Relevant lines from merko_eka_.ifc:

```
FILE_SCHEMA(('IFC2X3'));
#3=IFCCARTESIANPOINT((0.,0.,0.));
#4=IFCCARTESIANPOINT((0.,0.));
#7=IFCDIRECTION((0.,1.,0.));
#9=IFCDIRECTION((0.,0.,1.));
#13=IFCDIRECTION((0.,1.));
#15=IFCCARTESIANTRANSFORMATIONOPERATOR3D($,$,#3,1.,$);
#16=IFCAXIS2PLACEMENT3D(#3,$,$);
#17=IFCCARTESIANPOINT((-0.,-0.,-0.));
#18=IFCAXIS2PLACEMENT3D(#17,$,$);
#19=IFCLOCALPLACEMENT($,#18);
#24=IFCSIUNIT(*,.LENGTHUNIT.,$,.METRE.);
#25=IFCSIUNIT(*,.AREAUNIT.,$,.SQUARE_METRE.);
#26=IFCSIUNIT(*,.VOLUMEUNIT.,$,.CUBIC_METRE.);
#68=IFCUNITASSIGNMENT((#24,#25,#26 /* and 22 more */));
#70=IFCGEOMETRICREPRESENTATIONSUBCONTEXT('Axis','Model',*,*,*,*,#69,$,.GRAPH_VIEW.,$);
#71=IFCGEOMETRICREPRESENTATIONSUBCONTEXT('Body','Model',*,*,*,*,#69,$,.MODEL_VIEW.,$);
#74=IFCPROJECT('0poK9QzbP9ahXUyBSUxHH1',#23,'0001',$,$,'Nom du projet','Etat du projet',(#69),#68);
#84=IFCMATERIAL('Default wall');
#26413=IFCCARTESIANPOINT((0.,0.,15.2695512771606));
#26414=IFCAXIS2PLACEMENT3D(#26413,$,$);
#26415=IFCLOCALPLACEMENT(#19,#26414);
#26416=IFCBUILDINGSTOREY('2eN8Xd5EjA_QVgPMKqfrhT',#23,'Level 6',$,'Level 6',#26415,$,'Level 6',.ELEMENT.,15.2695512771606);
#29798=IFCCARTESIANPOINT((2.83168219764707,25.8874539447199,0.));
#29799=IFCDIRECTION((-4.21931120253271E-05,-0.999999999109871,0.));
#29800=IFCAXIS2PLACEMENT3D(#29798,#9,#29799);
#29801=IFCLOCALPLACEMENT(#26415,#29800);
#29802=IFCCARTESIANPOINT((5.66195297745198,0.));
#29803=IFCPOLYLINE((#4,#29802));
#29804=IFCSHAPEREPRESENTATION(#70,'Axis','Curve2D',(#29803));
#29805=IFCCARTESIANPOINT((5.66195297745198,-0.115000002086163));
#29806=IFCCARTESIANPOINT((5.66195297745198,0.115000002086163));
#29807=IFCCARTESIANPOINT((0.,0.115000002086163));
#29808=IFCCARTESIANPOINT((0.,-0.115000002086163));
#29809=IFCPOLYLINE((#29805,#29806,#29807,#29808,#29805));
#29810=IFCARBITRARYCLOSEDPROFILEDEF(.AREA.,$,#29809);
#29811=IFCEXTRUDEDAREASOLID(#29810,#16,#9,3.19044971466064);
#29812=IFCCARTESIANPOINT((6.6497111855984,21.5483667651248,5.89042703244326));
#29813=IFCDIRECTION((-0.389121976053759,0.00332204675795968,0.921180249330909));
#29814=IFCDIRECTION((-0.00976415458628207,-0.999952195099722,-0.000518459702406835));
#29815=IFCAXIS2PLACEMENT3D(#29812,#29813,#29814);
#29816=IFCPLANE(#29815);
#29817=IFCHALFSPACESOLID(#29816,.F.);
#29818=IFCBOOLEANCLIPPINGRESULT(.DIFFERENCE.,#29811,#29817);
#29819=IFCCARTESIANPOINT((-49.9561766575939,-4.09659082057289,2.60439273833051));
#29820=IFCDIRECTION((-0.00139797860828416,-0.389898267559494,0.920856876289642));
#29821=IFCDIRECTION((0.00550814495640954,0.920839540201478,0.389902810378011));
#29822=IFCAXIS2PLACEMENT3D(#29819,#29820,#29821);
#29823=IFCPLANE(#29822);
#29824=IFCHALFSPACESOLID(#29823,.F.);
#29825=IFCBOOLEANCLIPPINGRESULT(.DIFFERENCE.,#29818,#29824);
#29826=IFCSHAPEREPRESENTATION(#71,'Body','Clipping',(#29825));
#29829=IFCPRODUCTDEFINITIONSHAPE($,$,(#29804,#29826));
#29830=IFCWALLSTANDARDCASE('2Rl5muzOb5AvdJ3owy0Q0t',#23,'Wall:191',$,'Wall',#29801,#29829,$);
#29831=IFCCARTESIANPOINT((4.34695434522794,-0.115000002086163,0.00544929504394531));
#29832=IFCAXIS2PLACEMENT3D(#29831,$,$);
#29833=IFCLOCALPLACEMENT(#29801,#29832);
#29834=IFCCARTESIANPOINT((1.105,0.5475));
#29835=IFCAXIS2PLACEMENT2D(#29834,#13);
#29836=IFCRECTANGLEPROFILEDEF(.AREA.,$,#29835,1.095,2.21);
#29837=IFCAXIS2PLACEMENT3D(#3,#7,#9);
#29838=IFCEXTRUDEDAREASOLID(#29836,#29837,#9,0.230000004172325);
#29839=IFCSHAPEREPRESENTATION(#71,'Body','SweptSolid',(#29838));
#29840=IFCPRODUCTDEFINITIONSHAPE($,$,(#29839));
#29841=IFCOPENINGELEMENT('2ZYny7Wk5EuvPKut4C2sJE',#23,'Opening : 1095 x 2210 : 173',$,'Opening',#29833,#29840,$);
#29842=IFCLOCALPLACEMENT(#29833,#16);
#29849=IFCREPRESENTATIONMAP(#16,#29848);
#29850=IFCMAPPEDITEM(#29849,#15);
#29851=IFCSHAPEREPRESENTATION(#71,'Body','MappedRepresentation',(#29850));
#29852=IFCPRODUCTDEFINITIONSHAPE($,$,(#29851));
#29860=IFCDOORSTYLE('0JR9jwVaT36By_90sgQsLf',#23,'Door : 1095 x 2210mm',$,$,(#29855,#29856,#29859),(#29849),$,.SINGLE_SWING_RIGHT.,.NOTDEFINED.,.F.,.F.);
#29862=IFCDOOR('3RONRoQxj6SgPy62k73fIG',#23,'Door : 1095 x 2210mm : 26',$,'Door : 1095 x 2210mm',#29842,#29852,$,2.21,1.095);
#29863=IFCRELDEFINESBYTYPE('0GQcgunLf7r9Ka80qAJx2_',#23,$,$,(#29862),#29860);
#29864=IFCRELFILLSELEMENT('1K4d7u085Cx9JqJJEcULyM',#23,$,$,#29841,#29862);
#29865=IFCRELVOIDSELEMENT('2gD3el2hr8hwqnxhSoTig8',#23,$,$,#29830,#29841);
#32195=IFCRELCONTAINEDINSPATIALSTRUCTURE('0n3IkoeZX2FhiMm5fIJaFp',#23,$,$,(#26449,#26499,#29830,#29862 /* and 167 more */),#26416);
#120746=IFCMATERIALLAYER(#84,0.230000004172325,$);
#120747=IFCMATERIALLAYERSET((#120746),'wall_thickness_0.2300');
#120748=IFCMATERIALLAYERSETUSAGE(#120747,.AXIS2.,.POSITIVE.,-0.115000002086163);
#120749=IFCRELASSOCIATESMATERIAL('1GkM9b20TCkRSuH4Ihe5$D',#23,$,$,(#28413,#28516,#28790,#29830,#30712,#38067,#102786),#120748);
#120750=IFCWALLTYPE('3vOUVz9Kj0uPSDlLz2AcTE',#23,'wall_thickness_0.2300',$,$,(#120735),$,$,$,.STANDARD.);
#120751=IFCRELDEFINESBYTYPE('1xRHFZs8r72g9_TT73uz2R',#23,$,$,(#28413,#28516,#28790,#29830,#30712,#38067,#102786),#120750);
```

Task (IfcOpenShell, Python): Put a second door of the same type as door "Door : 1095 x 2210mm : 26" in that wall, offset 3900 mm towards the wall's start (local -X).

```python
import ifcopenshell
import ifcopenshell.api.feature
import ifcopenshell.api.geometry
import ifcopenshell.api.root
import ifcopenshell.geom
import ifcopenshell.util.element
import ifcopenshell.util.placement
import ifcopenshell.util.shape
import ifcopenshell.util.unit

model = ifcopenshell.open("merko_eka_.ifc")
unit_scale = ifcopenshell.util.unit.calculate_unit_scale(model)
settings = ifcopenshell.geom.settings()


def volume(element):
    """Net volume in cubic metres, openings subtracted."""
    shape = ifcopenshell.geom.create_shape(settings, element)
    return ifcopenshell.util.shape.get_volume(shape.geometry)


door = model.by_guid("3RONRoQxj6SgPy62k73fIG")
opening = door.FillsVoids[0].RelatingOpeningElement
wall = opening.VoidsElements[0].RelatingBuildingElement
before = volume(wall)
shift = ifcopenshell.util.placement.get_local_placement(wall.ObjectPlacement)[:3, 0] * -3.9 / unit_scale

# copy_class copies the void relationship, type, container and properties, but no geometry.
new_opening = ifcopenshell.api.root.copy_class(model, product=opening)
new_opening.Representation = ifcopenshell.util.element.copy_deep(
    model, opening.Representation, exclude=["IfcGeometricRepresentationContext", "IfcRepresentationMap"]
)
new_opening.Name = "Opening : 1095 x 2210"
new_door = ifcopenshell.api.root.copy_class(model, product=door)
new_door.Representation = ifcopenshell.util.element.copy_deep(
    model, door.Representation, exclude=["IfcGeometricRepresentationContext", "IfcRepresentationMap"]
)
new_door.Name = "Door : 1095 x 2210mm"
fills = ifcopenshell.api.feature.add_filling(model, opening=new_opening, element=new_door)
fills.OwnerHistory = new_door.OwnerHistory  # required in IFC2X3

for old, new in ((opening, new_opening), (door, new_door)):
    matrix = ifcopenshell.util.placement.get_local_placement(old.ObjectPlacement)
    matrix[:3, 3] += shift
    ifcopenshell.api.geometry.edit_object_placement(model, product=new, matrix=matrix, is_si=False)

after = volume(wall)

print(f"wall volume {before:.3f} -> {after:.3f} m3")

model.write("merko_eka__edited.ifc")
```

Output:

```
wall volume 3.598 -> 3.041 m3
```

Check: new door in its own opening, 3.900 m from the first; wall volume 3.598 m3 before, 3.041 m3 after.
